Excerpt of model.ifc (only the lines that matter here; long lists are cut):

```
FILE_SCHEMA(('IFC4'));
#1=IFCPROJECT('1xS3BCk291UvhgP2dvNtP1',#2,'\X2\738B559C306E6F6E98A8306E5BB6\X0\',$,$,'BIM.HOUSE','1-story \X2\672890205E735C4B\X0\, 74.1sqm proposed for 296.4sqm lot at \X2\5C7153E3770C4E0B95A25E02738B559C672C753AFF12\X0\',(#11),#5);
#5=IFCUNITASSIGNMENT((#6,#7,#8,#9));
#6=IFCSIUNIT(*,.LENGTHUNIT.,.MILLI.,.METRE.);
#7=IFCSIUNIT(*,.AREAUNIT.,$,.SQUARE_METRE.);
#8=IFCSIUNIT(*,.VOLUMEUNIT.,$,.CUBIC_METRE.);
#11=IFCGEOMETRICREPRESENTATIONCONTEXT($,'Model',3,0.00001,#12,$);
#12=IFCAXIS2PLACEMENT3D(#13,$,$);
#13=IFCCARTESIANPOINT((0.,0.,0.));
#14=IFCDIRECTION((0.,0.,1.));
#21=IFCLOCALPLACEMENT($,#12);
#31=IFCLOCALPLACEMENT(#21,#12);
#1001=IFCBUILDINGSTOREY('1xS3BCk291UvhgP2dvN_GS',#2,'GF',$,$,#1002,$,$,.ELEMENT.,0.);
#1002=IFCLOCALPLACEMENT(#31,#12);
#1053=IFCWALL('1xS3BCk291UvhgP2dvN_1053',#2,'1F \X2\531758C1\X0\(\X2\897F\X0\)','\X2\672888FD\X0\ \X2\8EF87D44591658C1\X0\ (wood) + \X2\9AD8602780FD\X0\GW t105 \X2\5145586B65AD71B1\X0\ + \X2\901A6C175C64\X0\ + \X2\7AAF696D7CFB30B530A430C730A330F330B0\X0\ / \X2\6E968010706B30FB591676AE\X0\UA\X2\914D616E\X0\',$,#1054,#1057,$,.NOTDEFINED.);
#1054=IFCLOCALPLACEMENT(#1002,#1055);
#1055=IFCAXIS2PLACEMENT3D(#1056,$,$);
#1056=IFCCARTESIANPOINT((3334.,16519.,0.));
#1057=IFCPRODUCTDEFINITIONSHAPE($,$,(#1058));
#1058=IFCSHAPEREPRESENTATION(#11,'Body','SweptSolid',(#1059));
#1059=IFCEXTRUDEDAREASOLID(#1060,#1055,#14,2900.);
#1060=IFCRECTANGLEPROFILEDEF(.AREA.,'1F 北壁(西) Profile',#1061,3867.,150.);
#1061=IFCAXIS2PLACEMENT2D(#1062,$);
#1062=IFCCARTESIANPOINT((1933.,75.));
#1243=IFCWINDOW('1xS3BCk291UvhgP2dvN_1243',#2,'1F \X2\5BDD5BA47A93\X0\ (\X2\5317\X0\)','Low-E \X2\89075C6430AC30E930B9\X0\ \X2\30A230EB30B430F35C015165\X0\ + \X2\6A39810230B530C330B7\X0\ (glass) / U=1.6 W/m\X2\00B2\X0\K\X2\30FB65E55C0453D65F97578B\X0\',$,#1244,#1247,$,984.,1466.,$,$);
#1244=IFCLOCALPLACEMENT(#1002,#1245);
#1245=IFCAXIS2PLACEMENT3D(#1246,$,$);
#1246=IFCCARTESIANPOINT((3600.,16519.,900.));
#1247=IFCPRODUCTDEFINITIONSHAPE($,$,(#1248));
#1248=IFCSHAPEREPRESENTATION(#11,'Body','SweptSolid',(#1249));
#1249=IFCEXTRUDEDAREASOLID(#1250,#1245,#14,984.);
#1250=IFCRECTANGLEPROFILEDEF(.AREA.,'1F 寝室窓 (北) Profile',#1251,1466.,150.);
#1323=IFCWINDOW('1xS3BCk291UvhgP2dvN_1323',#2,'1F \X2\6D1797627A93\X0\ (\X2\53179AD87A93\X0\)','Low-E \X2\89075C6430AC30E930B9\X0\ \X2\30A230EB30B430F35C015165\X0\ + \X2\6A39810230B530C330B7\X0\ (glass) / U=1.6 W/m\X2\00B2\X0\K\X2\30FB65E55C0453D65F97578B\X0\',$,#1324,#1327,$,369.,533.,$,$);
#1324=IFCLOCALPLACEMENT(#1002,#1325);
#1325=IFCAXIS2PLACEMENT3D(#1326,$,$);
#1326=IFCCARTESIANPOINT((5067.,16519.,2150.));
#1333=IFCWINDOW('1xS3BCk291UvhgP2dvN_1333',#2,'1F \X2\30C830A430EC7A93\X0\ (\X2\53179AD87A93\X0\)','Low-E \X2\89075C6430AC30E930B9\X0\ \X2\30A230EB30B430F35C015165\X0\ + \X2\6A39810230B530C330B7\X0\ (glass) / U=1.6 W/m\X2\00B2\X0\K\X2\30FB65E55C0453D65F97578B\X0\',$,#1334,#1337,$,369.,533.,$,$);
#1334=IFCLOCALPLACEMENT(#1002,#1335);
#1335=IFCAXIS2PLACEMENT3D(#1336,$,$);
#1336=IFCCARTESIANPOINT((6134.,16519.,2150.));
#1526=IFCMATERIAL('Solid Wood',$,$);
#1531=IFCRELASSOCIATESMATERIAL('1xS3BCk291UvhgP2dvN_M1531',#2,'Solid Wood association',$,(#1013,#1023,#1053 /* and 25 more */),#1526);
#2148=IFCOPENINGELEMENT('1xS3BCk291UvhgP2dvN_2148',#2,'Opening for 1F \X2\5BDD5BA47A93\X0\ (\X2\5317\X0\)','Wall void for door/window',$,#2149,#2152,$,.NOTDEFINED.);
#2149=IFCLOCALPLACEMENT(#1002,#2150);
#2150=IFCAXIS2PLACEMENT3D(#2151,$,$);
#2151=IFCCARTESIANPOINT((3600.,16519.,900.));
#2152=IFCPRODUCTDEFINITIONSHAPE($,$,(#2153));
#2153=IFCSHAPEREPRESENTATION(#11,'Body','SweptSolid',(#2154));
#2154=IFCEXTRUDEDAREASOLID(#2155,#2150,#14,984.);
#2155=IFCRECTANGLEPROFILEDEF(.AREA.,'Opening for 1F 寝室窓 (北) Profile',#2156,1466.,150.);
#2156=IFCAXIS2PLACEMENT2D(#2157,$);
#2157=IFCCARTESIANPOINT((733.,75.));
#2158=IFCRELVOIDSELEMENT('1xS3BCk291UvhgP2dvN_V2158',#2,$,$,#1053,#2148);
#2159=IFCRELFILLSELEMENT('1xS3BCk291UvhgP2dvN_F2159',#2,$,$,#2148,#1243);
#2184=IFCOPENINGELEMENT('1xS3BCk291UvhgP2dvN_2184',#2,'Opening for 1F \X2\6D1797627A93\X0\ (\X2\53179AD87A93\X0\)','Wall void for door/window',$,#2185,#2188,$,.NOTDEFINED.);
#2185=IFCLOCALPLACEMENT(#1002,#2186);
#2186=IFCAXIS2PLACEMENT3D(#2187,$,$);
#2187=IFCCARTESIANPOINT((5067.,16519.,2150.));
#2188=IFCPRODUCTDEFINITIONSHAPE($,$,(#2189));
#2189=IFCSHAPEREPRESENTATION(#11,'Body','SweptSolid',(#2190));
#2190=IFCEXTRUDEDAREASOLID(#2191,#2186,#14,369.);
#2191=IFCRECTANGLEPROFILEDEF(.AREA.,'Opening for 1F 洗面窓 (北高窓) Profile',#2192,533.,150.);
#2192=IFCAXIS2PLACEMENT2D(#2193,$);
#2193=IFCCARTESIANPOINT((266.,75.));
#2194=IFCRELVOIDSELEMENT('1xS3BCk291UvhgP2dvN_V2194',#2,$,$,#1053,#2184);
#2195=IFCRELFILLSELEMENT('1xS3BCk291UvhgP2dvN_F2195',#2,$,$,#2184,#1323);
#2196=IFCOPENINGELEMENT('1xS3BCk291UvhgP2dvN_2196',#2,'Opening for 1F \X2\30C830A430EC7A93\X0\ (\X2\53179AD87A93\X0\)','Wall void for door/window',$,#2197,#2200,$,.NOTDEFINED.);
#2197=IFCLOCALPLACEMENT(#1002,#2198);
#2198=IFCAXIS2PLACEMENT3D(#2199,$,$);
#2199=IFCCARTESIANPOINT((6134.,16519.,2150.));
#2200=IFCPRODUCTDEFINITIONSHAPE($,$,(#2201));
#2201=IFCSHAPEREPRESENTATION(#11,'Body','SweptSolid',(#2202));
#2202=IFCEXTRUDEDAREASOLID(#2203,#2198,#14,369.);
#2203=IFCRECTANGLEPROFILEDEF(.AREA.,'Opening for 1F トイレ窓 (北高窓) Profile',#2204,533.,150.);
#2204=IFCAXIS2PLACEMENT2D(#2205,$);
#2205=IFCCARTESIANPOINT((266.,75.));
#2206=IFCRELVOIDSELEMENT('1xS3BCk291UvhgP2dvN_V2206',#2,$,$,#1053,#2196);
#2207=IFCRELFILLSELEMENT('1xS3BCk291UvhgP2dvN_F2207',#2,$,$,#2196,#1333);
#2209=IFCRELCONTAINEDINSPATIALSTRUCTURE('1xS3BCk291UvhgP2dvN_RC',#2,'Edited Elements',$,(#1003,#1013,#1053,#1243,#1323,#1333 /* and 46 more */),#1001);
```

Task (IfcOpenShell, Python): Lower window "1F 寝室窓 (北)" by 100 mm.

```python
import numpy as np
import ifcopenshell
import ifcopenshell.api.geometry
import ifcopenshell.util.placement
import ifcopenshell.util.unit

model = ifcopenshell.open("model.ifc")
unit_scale = ifcopenshell.util.unit.calculate_unit_scale(model)

window = model.by_id(1243)
opening = window.FillsVoids[0].RelatingOpeningElement
dz = -100.0

shift = np.array([0.0, 0.0, dz])
# The window is not placed relative to its opening, so move both.
for product in (opening, window):
    matrix = ifcopenshell.util.placement.get_local_placement(product.ObjectPlacement)
    matrix[:3, 3] += shift
    ifcopenshell.api.geometry.edit_object_placement(model, product=product, matrix=matrix, is_si=False)

print(f"moved by {dz * unit_scale:+.3f} m")

model.write("model-out.ifc")
```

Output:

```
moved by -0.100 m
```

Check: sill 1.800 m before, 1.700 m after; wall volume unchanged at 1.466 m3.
